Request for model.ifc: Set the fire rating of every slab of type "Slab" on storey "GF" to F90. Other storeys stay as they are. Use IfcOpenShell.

First a look at what the model holds.

```python
import ifcopenshell
import ifcopenshell.util.element

model = ifcopenshell.open("model.ifc")
print(model.schema)
storey = next(s for s in model.by_type("IfcBuildingStorey") if s.Name == "GF")
slabs = [e for e in ifcopenshell.util.element.get_decomposition(storey) if e.is_a("IfcSlab")]
seen = {}
for e in slabs:
    element_type = ifcopenshell.util.element.get_type(e)
    key = (element_type.Name if element_type != e and element_type else None, ifcopenshell.util.element.get_pset(e, "Pset_SlabCommon", "FireRating"))
    seen[key] = seen.get(key, 0) + 1
for (name, value), count in sorted(seen.items(), key=str):
    print(count, "x", name, "|", value)
```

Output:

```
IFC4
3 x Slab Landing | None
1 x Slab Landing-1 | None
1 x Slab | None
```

```python
import ifcopenshell
import ifcopenshell.api.pset
import ifcopenshell.util.element

model = ifcopenshell.open("model.ifc")

storey = next(s for s in model.by_type("IfcBuildingStorey") if s.Name == "GF")
slabs = [e for e in ifcopenshell.util.element.get_decomposition(storey) if e.is_a("IfcSlab")]

count = 0
for e in slabs:
    element_type = ifcopenshell.util.element.get_type(e)
    if element_type in (None, e) or element_type.Name != "Slab":
        continue
    # add_pset returns the element's existing set when there is one.
    pset = ifcopenshell.api.pset.add_pset(model, product=e, name="Pset_SlabCommon")
    ifcopenshell.api.pset.edit_pset(model, pset=pset, properties={"FireRating": "F90"})
    count += 1

print(count, "slabs updated")

model.write("model_v2.ifc")
```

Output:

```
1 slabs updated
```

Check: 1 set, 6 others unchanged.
